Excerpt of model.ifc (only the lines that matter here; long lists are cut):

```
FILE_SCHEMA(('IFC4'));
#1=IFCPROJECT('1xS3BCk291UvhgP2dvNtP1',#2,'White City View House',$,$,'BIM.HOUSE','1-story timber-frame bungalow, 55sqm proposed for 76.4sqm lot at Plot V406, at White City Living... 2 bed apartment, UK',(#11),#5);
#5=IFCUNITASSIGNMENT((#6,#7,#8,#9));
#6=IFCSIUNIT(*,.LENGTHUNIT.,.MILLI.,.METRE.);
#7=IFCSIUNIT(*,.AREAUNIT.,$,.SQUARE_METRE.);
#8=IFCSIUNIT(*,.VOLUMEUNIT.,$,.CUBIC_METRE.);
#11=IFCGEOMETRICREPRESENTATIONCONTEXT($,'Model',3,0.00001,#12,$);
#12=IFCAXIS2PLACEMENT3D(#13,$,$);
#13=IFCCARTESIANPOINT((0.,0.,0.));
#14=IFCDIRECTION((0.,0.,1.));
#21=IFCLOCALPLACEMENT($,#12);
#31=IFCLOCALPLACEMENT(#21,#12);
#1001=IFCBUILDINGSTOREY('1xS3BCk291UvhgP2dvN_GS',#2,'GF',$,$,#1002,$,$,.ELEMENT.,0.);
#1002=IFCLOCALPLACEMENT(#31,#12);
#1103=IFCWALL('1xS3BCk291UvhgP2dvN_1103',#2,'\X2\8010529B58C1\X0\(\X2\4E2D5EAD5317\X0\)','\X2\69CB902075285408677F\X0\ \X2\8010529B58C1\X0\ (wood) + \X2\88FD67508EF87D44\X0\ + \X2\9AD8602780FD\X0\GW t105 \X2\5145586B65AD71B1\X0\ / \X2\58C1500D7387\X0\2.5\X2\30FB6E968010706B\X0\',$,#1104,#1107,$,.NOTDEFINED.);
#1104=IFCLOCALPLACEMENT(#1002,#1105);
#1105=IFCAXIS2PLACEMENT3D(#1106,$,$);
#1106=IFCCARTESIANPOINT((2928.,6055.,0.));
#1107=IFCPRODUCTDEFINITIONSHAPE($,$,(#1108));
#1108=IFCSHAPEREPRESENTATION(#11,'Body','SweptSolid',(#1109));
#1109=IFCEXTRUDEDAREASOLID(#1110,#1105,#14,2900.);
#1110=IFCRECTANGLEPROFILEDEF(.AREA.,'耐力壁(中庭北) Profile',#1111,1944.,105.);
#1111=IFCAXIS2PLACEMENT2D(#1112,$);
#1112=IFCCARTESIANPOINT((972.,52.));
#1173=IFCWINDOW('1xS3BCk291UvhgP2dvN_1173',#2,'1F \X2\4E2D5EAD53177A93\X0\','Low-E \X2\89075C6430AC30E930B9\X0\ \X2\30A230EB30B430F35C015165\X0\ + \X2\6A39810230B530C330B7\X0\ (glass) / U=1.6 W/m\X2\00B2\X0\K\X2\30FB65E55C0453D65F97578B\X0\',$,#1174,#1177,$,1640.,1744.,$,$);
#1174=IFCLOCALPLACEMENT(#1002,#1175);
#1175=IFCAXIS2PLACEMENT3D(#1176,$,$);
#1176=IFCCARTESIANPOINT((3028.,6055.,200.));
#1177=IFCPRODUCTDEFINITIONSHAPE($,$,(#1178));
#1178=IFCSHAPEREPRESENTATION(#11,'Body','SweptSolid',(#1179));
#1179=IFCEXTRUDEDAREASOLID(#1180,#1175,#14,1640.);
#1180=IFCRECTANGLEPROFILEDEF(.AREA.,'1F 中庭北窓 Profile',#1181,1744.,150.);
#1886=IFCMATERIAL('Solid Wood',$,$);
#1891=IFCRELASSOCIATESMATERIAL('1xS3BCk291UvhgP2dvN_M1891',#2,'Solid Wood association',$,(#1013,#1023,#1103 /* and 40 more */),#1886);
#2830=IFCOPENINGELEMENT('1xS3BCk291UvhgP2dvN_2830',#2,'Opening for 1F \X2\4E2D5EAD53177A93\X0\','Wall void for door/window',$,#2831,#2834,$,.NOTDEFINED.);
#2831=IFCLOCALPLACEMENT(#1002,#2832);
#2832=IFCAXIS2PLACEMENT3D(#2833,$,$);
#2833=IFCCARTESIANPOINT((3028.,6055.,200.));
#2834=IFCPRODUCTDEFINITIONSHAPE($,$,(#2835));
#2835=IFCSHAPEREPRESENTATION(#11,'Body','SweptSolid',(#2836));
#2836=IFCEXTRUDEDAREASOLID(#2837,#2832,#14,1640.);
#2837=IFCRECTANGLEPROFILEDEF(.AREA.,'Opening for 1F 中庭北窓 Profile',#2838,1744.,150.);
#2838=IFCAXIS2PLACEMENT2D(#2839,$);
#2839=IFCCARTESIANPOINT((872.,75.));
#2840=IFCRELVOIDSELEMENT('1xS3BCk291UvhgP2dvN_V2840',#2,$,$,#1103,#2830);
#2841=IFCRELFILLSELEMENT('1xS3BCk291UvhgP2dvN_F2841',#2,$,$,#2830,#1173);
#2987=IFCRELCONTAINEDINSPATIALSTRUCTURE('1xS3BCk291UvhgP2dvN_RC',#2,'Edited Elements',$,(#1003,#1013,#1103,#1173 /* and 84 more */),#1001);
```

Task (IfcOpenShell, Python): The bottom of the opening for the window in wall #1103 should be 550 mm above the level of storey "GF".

```python
import numpy as np
import ifcopenshell
import ifcopenshell.api.geometry
import ifcopenshell.geom
import ifcopenshell.util.element
import ifcopenshell.util.placement
import ifcopenshell.util.shape
import ifcopenshell.util.unit

model = ifcopenshell.open("model.ifc")
unit_scale = ifcopenshell.util.unit.calculate_unit_scale(model)

window = model.by_guid("1xS3BCk291UvhgP2dvN_1173")
opening = window.FillsVoids[0].RelatingOpeningElement
storey = ifcopenshell.util.element.get_container(window, ifc_class="IfcBuildingStorey")
level = ifcopenshell.util.placement.get_local_placement(storey.ObjectPlacement)[2, 3]

# The opening's origin need not be at the sill, so measure its lowest point.
shape = ifcopenshell.geom.create_shape(ifcopenshell.geom.settings(), opening)
bottom = ifcopenshell.util.shape.get_shape_bottom_elevation(shape, shape.geometry) / unit_scale
dz = level + 550.0 - bottom

shift = np.array([0.0, 0.0, dz])
# The window is not placed relative to its opening, so move both.
for product in (opening, window):
    matrix = ifcopenshell.util.placement.get_local_placement(product.ObjectPlacement)
    matrix[:3, 3] += shift
    ifcopenshell.api.geometry.edit_object_placement(model, product=product, matrix=matrix, is_si=False)

print(f"moved by {dz * unit_scale:+.3f} m")

model.write("model_updated.ifc")
```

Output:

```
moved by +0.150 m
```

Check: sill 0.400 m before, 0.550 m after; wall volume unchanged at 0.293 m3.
